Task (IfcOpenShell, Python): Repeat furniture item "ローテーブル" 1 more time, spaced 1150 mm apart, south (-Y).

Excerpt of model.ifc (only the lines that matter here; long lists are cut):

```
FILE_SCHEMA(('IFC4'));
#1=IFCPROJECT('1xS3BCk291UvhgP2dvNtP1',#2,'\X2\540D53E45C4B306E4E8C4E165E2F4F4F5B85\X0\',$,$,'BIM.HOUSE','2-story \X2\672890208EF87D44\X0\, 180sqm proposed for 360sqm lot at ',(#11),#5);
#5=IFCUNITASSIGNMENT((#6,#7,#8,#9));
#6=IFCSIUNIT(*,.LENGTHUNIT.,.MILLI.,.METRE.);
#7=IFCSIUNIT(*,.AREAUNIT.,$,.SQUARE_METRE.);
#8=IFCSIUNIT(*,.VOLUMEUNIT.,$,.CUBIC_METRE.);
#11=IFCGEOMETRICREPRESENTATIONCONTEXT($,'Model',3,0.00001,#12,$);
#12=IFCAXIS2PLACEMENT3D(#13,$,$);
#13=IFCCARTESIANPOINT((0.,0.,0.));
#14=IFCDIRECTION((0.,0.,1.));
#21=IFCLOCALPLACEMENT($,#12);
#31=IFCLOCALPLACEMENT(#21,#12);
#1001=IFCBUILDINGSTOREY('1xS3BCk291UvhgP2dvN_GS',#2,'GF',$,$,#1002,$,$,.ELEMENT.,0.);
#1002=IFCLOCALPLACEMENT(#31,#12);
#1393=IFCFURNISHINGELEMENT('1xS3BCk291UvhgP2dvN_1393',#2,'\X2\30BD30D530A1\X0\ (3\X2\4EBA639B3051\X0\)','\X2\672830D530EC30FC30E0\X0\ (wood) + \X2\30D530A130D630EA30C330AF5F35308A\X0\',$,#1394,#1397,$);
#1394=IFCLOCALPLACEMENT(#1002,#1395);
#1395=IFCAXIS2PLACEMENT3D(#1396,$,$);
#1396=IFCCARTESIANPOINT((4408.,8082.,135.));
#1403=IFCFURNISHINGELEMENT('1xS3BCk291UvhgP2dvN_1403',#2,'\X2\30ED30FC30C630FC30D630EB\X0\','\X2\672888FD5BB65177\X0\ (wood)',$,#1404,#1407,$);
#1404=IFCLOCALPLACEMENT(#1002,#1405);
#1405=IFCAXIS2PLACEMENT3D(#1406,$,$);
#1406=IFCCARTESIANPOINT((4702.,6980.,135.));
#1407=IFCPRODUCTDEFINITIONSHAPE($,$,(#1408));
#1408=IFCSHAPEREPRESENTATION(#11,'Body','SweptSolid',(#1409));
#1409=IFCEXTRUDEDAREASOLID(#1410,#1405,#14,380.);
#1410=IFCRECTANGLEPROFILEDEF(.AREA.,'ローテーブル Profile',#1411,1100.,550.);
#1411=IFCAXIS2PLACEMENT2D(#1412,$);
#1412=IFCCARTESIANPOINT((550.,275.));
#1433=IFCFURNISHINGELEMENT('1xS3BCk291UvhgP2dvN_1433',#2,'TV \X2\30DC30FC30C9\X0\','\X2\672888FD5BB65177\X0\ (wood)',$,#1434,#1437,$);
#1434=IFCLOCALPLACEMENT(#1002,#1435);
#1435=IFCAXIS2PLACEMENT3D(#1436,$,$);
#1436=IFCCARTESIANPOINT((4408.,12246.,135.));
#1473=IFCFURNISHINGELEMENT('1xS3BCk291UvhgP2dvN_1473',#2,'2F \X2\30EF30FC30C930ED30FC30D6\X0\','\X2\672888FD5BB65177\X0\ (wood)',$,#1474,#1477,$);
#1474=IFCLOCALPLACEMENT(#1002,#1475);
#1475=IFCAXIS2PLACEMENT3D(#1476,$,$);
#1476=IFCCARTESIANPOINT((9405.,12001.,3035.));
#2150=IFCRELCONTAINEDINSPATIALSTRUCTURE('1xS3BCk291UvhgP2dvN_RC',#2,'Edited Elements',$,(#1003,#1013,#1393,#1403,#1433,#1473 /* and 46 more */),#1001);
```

```python
import numpy as np
import ifcopenshell
import ifcopenshell.api.geometry
import ifcopenshell.api.root
import ifcopenshell.util.element
import ifcopenshell.util.placement
import ifcopenshell.util.unit

model = ifcopenshell.open("model.ifc")
unit_scale = ifcopenshell.util.unit.calculate_unit_scale(model)


def reuse_history(source, copy):
    """copy_class also copies each property set's owner history, people and application; keep the originals."""
    for rel in copy.IsDefinedBy:
        if rel.is_a("IfcRelDefinesByProperties") and (history := rel.RelatingPropertyDefinition.OwnerHistory):
            rel.RelatingPropertyDefinition.OwnerHistory = source.OwnerHistory
            ifcopenshell.util.element.remove_deep2(model, history)


source = model.by_id(1403)
base = ifcopenshell.util.placement.get_local_placement(source.ObjectPlacement)
step = np.array([0.0, -1.0, 0.0]) * 1.15 / unit_scale

for i in range(1, 2):
    copy = ifcopenshell.api.root.copy_class(model, product=source)
    copy.Representation = ifcopenshell.util.element.copy_deep(
        model, source.Representation, exclude=["IfcGeometricRepresentationContext", "IfcRepresentationMap"]
    )
    reuse_history(source, copy)
    matrix = base.copy()
    matrix[:3, 3] += i * step
    print("added at", matrix[:3, 3].round(3) + 0.0)
    ifcopenshell.api.geometry.edit_object_placement(model, product=copy, matrix=matrix, is_si=False)

model.write("model_rev.ifc")
```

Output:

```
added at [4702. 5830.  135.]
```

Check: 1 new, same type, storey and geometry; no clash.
